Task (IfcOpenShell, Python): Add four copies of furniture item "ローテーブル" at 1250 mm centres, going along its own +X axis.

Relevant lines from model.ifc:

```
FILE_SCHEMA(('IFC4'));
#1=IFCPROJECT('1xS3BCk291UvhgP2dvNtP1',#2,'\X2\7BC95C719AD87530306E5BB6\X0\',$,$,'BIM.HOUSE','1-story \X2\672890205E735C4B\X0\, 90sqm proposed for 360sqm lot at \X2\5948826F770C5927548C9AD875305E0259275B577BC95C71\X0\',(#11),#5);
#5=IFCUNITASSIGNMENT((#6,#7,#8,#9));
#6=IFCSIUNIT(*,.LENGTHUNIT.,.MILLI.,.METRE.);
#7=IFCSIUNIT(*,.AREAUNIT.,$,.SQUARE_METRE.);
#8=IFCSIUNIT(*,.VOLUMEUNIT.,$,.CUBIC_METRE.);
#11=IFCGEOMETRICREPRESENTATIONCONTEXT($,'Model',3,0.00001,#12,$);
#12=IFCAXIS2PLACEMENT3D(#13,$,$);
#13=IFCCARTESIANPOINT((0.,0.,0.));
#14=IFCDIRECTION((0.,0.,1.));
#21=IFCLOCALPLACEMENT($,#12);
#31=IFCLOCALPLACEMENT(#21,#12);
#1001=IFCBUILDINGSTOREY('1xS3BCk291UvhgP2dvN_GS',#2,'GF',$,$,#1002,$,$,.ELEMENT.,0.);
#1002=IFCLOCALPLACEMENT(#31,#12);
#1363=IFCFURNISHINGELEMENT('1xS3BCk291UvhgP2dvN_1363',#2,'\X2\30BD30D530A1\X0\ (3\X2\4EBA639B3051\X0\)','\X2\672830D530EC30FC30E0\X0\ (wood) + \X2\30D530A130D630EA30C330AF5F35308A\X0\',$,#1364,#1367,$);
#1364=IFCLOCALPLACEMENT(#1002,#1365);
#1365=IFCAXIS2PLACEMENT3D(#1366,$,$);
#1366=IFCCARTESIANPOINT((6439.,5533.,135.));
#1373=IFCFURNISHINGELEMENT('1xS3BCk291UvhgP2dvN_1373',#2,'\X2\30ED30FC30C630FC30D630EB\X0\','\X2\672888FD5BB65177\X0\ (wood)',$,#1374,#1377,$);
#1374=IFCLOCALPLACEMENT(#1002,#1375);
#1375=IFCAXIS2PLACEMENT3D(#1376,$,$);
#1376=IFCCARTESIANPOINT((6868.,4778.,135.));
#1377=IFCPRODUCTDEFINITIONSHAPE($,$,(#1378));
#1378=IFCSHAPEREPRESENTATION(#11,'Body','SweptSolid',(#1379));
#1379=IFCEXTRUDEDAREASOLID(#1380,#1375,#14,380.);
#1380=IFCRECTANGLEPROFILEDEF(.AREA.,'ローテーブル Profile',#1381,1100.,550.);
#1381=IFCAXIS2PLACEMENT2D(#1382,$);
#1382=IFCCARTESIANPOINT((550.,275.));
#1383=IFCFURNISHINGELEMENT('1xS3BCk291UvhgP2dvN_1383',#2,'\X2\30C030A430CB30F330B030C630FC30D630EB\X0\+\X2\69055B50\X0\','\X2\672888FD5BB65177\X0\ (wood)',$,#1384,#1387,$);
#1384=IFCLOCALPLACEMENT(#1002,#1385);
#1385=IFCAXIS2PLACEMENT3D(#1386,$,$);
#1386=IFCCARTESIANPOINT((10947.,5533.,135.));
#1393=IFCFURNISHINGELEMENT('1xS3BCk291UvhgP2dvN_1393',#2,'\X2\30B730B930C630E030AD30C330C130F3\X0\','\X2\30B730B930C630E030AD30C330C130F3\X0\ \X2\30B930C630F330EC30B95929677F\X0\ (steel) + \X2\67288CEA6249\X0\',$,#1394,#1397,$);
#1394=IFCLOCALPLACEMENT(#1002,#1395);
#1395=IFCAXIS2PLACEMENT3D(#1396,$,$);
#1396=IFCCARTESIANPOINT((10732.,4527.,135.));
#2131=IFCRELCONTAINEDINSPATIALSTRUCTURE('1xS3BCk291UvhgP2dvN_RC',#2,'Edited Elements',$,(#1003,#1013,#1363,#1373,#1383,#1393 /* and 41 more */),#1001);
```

```python
import ifcopenshell
import ifcopenshell.api.geometry
import ifcopenshell.api.root
import ifcopenshell.util.element
import ifcopenshell.util.placement
import ifcopenshell.util.unit

model = ifcopenshell.open("model.ifc")
unit_scale = ifcopenshell.util.unit.calculate_unit_scale(model)


def reuse_history(source, copy):
    """copy_class also copies each property set's owner history, people and application; keep the originals."""
    for rel in copy.IsDefinedBy:
        if rel.is_a("IfcRelDefinesByProperties") and (history := rel.RelatingPropertyDefinition.OwnerHistory):
            rel.RelatingPropertyDefinition.OwnerHistory = source.OwnerHistory
            ifcopenshell.util.element.remove_deep2(model, history)


source = model.by_id(1373)
base = ifcopenshell.util.placement.get_local_placement(source.ObjectPlacement)
step = base[:3, 0] * 1.25 / unit_scale

for i in range(1, 5):
    copy = ifcopenshell.api.root.copy_class(model, product=source)
    copy.Representation = ifcopenshell.util.element.copy_deep(
        model, source.Representation, exclude=["IfcGeometricRepresentationContext", "IfcRepresentationMap"]
    )
    reuse_history(source, copy)
    matrix = base.copy()
    matrix[:3, 3] += i * step
    print("added at", matrix[:3, 3].round(3) + 0.0)
    ifcopenshell.api.geometry.edit_object_placement(model, product=copy, matrix=matrix, is_si=False)

model.write("model-out.ifc")
```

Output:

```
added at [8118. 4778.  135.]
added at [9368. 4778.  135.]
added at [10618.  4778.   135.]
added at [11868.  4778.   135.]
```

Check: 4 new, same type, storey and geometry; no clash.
